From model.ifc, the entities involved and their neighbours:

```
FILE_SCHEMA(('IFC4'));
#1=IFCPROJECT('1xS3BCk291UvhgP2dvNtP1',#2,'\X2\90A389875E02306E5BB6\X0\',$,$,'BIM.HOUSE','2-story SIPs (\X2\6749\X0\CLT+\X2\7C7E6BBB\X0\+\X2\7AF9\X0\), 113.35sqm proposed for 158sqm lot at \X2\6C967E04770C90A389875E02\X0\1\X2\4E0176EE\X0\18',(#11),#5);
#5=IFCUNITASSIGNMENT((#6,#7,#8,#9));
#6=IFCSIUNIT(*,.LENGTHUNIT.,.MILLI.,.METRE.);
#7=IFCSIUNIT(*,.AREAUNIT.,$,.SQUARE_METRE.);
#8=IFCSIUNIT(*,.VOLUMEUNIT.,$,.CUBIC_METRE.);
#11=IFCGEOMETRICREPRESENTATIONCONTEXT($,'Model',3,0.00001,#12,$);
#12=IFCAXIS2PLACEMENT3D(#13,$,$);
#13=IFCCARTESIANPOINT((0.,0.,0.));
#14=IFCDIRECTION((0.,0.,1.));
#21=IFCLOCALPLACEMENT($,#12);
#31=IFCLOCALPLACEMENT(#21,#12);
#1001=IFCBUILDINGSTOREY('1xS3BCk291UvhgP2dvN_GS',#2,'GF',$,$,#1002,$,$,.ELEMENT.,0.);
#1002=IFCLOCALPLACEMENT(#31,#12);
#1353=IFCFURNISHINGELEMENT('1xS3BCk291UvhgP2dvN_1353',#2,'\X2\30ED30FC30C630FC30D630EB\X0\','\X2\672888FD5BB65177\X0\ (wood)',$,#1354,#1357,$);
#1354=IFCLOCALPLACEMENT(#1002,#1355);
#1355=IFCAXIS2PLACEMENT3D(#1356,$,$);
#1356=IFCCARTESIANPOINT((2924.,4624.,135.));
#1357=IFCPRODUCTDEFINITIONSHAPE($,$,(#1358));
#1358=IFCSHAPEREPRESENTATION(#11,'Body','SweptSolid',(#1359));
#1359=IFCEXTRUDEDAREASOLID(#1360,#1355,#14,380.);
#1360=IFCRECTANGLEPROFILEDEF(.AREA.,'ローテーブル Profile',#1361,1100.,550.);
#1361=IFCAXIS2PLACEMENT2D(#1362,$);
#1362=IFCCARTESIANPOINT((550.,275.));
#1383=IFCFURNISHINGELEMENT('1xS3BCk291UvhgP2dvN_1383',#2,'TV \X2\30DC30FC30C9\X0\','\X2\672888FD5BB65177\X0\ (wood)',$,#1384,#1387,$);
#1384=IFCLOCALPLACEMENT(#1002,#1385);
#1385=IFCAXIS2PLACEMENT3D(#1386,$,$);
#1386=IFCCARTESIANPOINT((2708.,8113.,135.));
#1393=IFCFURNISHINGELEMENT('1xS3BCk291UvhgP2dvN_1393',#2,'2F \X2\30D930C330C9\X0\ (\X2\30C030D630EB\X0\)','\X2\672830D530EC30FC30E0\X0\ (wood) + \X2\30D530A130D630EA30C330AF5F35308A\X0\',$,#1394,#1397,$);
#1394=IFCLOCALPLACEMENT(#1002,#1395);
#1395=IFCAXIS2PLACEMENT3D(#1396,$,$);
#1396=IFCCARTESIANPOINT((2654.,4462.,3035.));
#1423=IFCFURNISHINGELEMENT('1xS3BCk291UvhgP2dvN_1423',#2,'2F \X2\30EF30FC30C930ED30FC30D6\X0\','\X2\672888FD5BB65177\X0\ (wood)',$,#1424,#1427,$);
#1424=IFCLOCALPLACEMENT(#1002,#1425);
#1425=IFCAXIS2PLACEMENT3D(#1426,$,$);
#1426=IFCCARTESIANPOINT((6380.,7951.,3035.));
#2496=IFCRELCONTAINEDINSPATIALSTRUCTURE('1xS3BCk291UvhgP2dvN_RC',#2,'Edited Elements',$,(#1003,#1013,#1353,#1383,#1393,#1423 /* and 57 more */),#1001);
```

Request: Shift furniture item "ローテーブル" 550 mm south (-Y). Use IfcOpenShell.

```python
import ifcopenshell
import ifcopenshell.api.geometry
import ifcopenshell.util.placement
import ifcopenshell.util.unit

model = ifcopenshell.open("model.ifc")
unit_scale = ifcopenshell.util.unit.calculate_unit_scale(model)

item = model.by_id(1353)
matrix = ifcopenshell.util.placement.get_local_placement(item.ObjectPlacement)
matrix[1, 3] -= 0.55 / unit_scale
ifcopenshell.api.geometry.edit_object_placement(model, product=item, matrix=matrix, is_si=False)

print(ifcopenshell.util.placement.get_local_placement(item.ObjectPlacement).round(3) + 0.0)

model.write("model_updated.ifc")
```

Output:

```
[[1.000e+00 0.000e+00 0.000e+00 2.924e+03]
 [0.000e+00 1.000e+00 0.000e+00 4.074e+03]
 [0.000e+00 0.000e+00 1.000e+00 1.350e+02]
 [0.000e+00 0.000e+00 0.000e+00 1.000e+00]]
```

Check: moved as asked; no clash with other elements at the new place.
